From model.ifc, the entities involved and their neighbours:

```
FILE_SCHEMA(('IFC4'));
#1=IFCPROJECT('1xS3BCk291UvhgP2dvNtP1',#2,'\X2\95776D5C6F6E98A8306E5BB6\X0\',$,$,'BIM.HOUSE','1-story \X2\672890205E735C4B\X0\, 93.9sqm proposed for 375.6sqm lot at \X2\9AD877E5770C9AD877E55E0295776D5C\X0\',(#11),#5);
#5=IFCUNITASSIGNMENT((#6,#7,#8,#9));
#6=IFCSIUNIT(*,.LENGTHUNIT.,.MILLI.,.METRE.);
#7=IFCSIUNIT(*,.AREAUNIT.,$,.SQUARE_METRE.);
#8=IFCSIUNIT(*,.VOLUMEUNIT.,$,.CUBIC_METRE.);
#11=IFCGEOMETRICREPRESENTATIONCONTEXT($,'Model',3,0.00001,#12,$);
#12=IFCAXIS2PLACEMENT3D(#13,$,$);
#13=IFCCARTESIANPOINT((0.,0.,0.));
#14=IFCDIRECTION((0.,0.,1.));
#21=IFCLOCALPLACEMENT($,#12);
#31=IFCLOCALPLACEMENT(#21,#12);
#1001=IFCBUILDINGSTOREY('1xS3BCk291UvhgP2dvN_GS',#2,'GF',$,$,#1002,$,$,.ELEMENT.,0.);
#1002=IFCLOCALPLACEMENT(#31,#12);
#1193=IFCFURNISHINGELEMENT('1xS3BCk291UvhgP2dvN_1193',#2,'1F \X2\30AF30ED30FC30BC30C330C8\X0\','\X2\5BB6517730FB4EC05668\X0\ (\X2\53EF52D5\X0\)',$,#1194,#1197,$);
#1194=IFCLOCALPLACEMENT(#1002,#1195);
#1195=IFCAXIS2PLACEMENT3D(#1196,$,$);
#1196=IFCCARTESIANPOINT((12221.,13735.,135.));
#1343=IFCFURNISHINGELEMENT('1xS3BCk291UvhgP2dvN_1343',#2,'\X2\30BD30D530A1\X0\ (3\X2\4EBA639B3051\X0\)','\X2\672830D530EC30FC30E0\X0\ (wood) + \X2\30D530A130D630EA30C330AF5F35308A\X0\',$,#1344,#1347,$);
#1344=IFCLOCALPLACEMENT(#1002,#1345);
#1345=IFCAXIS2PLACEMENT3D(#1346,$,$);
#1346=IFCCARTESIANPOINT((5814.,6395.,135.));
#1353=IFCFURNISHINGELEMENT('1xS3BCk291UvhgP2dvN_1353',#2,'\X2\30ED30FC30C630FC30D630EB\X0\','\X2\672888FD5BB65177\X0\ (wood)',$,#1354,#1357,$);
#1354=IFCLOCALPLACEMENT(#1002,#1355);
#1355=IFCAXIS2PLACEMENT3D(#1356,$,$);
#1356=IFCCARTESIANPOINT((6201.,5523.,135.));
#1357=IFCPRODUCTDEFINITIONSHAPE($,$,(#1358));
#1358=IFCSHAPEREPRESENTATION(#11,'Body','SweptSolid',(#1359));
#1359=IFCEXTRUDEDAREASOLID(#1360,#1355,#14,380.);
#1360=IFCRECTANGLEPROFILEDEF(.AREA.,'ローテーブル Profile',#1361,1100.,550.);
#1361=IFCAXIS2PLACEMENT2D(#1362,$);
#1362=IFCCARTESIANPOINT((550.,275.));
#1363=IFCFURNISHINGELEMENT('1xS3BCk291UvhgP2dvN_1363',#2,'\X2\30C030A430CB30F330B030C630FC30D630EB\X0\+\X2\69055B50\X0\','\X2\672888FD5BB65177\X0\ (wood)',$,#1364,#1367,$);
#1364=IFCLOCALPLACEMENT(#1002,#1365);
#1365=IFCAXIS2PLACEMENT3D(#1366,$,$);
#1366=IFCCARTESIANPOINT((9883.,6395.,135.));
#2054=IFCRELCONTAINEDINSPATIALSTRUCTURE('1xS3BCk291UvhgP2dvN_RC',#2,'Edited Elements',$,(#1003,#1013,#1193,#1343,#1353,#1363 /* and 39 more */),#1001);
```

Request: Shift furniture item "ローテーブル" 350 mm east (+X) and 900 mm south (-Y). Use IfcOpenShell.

```python
import ifcopenshell
import ifcopenshell.api.geometry
import ifcopenshell.util.placement

model = ifcopenshell.open("model.ifc")

item = model.by_guid("1xS3BCk291UvhgP2dvN_1353")
matrix = ifcopenshell.util.placement.get_local_placement(item.ObjectPlacement)
matrix[0, 3] += 350.0
matrix[1, 3] -= 900.0
ifcopenshell.api.geometry.edit_object_placement(model, product=item, matrix=matrix, is_si=False)

print(ifcopenshell.util.placement.get_local_placement(item.ObjectPlacement).round(3) + 0.0)

model.write("model_updated.ifc")
```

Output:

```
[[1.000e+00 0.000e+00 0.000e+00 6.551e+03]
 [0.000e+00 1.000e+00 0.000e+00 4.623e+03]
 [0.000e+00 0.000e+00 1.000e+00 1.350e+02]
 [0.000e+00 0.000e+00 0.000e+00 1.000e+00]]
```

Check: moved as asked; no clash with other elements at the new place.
